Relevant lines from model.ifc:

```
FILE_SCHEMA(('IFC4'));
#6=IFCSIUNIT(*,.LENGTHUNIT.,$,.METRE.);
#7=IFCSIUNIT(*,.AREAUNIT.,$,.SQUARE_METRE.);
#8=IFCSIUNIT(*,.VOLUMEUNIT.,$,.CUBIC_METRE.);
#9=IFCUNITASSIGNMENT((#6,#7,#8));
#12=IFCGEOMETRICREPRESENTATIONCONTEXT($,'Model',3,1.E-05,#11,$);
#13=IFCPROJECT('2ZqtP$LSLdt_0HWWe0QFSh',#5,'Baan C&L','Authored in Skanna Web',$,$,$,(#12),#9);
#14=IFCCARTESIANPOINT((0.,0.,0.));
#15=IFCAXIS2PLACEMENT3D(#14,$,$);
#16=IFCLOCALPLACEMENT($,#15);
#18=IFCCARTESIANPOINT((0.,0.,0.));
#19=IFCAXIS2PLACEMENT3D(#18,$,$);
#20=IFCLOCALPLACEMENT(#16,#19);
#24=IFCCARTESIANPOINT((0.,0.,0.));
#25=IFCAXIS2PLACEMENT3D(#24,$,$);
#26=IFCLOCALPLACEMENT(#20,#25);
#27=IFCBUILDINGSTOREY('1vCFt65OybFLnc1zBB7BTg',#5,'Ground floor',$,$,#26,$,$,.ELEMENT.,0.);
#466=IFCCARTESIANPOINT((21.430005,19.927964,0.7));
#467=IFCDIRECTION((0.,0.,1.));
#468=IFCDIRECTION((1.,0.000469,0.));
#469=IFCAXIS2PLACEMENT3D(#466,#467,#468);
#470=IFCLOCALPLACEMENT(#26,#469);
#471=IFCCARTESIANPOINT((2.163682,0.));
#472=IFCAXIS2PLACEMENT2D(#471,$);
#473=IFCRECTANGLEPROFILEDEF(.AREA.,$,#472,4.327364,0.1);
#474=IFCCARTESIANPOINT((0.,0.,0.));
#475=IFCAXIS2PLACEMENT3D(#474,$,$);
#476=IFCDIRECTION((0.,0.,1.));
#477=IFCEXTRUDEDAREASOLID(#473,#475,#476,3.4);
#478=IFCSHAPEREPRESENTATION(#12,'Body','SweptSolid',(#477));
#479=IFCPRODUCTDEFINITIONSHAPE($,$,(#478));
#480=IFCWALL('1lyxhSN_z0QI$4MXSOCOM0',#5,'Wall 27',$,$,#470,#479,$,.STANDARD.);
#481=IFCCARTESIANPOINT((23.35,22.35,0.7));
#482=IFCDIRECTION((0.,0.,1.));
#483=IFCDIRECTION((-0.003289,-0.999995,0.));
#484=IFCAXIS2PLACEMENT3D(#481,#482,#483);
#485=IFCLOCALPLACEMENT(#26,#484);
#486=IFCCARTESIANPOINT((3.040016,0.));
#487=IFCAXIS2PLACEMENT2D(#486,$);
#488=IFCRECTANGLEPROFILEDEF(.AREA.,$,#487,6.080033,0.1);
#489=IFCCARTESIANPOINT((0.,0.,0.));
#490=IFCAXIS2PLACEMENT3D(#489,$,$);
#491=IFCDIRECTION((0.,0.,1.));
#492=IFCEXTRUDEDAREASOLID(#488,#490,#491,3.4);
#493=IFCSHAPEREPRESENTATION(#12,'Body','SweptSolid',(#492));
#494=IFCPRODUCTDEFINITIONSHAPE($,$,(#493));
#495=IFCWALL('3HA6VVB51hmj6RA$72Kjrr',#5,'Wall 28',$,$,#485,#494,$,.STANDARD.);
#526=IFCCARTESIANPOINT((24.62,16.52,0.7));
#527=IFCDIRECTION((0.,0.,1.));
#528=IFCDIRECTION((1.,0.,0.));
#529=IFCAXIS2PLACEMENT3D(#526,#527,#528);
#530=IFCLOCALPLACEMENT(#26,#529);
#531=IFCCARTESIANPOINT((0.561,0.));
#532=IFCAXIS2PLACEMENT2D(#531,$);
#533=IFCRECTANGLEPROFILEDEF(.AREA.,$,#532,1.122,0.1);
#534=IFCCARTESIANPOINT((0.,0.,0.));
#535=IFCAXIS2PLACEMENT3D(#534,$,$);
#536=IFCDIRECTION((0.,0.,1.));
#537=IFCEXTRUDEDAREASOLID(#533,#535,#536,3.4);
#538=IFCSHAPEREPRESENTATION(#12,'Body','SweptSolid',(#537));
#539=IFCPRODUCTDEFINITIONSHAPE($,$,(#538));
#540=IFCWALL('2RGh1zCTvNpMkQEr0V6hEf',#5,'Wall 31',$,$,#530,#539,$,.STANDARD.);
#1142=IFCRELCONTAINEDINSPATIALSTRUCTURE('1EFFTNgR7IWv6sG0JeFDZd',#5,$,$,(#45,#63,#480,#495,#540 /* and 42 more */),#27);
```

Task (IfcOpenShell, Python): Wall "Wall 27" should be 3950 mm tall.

```python
import ifcopenshell
import ifcopenshell.geom
import ifcopenshell.util.shape

model = ifcopenshell.open("model.ifc")
settings = ifcopenshell.geom.settings()


def volume(element):
    """Net volume in cubic metres, openings subtracted."""
    shape = ifcopenshell.geom.create_shape(settings, element)
    return ifcopenshell.util.shape.get_volume(shape.geometry)


wall = model.by_guid("1lyxhSN_z0QI$4MXSOCOM0")
before = volume(wall)

body = next(r for r in wall.Representation.Representations if r.RepresentationIdentifier == "Body")
solid = body.Items[0]
old_height = solid.Depth
solid.Depth = 3.95
after = volume(wall)

print(f"height {old_height:g} -> {solid.Depth:g}, volume {before:.3f} -> {after:.3f} m3")

model.write("model_rev.ifc")
```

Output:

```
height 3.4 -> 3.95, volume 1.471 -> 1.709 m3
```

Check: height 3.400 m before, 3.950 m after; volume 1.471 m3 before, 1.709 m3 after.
